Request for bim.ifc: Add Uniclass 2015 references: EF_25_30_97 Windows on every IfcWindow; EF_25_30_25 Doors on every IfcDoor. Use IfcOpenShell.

First a look at what the model holds.

```python
import ifcopenshell

model = ifcopenshell.open("bim.ifc")
print(model.schema)
print("classifications:", [c.Name for c in model.by_type("IfcClassification")])
for ifc_class in ("IfcDoor", "IfcRoof", "IfcStair", "IfcWall", "IfcWindow"):
    print(ifc_class, len(model.by_type(ifc_class)))
```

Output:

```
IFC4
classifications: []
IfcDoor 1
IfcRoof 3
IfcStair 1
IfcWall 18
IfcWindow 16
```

```python
import ifcopenshell
import ifcopenshell.api.classification

model = ifcopenshell.open("bim.ifc")

system = ifcopenshell.api.classification.add_classification(model, classification="Uniclass 2015")

codes = {
    "IfcWindow": ("EF_25_30_97", "Windows"),
    "IfcDoor": ("EF_25_30_25", "Doors"),
}
for ifc_class, (code, name) in codes.items():
    products = model.by_type(ifc_class)
    ifcopenshell.api.classification.add_reference(
        model, products=products, classification=system, identification=code, name=name
    )
    print(code, len(products))

model.write("bim_updated.ifc")
```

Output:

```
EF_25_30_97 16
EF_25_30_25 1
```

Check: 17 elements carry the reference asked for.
